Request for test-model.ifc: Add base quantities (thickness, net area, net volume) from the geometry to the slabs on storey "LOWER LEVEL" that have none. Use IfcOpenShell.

First a look at what the model holds.

```python
import ifcopenshell
import ifcopenshell.util.element
import ifcopenshell.util.unit

model = ifcopenshell.open("test-model.ifc")
print(model.schema)
for unit_type in ("LENGTHUNIT", "AREAUNIT", "VOLUMEUNIT"):
    print(unit_type, ifcopenshell.util.unit.calculate_unit_scale(model, unit_type))
storey = next(s for s in model.by_type("IfcBuildingStorey") if s.Name == "LOWER LEVEL")
slabs = [e for e in ifcopenshell.util.element.get_decomposition(storey) if e.is_a("IfcSlab")]
for e in sorted(slabs, key=lambda e: e.id()):
    print(e.id(), e.is_a(), e.Name, list(ifcopenshell.util.element.get_psets(e, qtos_only=True)), sep=" | ")
```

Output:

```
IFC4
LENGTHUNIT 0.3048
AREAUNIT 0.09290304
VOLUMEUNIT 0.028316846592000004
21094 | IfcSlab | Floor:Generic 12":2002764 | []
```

```python
import ifcopenshell
import ifcopenshell.api.pset
import ifcopenshell.geom
import ifcopenshell.util.element
import ifcopenshell.util.shape
import ifcopenshell.util.unit

model = ifcopenshell.open("test-model.ifc")
unit_scale = ifcopenshell.util.unit.calculate_unit_scale(model)
area_scale = ifcopenshell.util.unit.calculate_unit_scale(model, "AREAUNIT")
volume_scale = ifcopenshell.util.unit.calculate_unit_scale(model, "VOLUMEUNIT")
settings = ifcopenshell.geom.settings()

storey = next(s for s in model.by_type("IfcBuildingStorey") if s.Name == "LOWER LEVEL")
slabs = [e for e in ifcopenshell.util.element.get_decomposition(storey) if e.is_a("IfcSlab")]

for e in sorted(slabs, key=lambda e: e.id()):
    if ifcopenshell.util.element.get_psets(e, qtos_only=True, should_inherit=False):
        continue
    # Geometry comes back in metres, in the element's own axes.
    shape = ifcopenshell.geom.create_shape(settings, e)
    values = {
        "Width": ifcopenshell.util.shape.get_z(shape.geometry) / unit_scale,
        "NetArea": ifcopenshell.util.shape.get_footprint_area(shape.geometry) / area_scale,
        "NetVolume": ifcopenshell.util.shape.get_volume(shape.geometry) / volume_scale,
    }
    qto = ifcopenshell.api.pset.add_qto(model, product=e, name="Qto_SlabBaseQuantities")
    ifcopenshell.api.pset.edit_qto(model, qto=qto, properties=values)
    print(e.id(), {k: round(v, 3) for k, v in values.items()})

model.write("test-model_edited.ifc")
```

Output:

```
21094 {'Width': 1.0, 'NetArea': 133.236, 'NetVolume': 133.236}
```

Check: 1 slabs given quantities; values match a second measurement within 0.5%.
